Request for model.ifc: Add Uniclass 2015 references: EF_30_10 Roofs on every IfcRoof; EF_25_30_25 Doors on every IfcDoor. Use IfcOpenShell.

First a look at what the model holds.

```python
import ifcopenshell

model = ifcopenshell.open("model.ifc")
print(model.schema)
print("classifications:", [c.Name for c in model.by_type("IfcClassification")])
for ifc_class in ("IfcDoor", "IfcRoof", "IfcStair", "IfcWall", "IfcWindow"):
    print(ifc_class, len(model.by_type(ifc_class)))
```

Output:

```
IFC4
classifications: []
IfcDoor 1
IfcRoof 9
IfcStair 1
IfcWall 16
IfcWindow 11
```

```python
import ifcopenshell
import ifcopenshell.api.classification

model = ifcopenshell.open("model.ifc")

system = ifcopenshell.api.classification.add_classification(model, classification="Uniclass 2015")

codes = {
    "IfcRoof": ("EF_30_10", "Roofs"),
    "IfcDoor": ("EF_25_30_25", "Doors"),
}
for ifc_class, (code, name) in codes.items():
    products = model.by_type(ifc_class)
    ifcopenshell.api.classification.add_reference(
        model, products=products, classification=system, identification=code, name=name
    )
    print(code, len(products))

model.write("model-out.ifc")
```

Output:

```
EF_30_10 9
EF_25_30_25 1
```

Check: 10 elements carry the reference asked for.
